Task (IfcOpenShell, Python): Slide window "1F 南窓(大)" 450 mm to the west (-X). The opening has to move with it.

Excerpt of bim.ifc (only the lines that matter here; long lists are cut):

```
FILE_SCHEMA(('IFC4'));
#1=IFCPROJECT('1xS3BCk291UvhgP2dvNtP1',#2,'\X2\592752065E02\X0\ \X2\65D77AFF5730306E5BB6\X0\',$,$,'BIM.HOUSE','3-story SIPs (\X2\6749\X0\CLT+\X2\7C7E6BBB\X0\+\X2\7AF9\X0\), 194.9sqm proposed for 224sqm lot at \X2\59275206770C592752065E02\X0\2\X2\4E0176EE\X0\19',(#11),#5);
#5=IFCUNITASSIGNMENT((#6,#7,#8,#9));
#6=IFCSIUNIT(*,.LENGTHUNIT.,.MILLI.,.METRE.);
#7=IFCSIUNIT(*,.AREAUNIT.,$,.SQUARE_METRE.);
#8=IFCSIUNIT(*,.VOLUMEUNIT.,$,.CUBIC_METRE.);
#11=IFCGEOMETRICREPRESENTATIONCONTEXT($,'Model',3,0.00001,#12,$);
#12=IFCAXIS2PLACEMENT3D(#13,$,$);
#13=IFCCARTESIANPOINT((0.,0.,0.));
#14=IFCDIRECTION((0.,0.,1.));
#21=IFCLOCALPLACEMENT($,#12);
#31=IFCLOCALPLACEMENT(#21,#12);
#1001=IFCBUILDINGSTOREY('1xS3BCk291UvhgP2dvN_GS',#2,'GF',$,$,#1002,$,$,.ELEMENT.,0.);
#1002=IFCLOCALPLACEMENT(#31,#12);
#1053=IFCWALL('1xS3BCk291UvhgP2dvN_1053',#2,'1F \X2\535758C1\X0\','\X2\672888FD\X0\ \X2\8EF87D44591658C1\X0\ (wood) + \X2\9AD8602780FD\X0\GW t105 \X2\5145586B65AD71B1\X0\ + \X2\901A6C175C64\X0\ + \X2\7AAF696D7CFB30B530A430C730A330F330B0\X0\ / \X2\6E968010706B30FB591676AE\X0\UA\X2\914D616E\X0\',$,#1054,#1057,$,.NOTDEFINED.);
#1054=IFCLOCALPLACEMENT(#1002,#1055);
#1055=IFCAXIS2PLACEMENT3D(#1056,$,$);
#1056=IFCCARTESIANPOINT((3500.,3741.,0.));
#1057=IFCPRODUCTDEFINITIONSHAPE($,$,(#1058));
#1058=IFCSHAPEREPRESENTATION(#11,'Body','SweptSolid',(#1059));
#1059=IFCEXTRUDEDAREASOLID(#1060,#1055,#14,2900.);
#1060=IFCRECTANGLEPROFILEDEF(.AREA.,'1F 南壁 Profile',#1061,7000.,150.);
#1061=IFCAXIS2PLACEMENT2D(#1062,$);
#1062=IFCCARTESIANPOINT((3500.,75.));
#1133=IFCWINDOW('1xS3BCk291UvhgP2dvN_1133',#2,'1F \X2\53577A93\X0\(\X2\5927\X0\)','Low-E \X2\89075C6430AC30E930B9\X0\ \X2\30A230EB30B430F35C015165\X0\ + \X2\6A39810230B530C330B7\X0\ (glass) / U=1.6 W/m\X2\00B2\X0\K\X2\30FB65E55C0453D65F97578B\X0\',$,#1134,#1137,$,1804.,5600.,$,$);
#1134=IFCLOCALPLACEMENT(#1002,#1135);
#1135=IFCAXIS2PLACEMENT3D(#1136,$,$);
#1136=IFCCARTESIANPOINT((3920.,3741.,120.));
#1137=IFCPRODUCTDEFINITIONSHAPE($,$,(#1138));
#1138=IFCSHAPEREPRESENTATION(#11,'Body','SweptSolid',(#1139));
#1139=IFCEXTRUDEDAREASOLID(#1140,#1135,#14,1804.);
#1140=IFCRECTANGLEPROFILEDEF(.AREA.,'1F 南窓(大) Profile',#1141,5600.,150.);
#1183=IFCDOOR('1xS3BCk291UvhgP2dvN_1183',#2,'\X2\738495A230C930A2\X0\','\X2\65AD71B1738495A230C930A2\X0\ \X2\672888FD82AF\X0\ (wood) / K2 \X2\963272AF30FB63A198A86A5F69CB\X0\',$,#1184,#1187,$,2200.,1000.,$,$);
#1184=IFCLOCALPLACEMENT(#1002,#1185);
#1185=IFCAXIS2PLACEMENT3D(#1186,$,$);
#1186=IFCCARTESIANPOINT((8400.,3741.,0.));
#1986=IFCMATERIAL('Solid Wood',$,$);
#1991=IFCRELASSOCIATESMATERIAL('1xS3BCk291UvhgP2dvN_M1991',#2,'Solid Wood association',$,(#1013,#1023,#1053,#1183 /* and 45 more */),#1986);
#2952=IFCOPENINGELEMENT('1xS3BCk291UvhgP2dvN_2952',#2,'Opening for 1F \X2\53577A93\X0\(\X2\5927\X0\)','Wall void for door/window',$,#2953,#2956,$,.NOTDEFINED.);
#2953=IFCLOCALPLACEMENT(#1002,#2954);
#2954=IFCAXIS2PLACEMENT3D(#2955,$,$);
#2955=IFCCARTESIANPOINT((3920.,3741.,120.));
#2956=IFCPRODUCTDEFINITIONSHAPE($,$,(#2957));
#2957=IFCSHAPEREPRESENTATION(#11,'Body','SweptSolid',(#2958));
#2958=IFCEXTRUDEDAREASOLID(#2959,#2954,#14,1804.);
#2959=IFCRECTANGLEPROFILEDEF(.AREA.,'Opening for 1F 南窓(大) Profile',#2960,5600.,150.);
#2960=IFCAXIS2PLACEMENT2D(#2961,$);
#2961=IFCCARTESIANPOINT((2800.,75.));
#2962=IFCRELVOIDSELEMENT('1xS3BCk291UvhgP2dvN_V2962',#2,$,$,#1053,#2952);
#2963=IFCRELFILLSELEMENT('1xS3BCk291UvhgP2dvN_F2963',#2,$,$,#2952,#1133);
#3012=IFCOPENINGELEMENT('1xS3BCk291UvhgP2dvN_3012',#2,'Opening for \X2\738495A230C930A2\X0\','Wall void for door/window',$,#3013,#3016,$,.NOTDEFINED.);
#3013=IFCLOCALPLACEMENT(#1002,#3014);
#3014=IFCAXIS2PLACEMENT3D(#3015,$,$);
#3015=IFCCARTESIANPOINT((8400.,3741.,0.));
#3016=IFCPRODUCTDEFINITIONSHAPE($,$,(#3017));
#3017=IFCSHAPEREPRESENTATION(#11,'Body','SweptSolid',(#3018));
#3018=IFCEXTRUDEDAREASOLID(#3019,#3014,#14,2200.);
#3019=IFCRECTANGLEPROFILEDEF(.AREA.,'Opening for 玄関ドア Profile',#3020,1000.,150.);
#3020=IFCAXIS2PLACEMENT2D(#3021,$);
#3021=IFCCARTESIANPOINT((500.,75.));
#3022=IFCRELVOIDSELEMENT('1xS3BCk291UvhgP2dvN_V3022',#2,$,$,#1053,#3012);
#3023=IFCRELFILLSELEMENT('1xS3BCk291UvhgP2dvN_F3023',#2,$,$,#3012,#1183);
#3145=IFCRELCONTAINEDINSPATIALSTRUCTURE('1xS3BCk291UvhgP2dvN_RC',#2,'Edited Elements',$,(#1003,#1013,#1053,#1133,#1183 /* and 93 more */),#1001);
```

```python
import ifcopenshell
import ifcopenshell.api.geometry
import ifcopenshell.util.placement
import ifcopenshell.util.unit

model = ifcopenshell.open("bim.ifc")
unit_scale = ifcopenshell.util.unit.calculate_unit_scale(model)

window = model.by_guid("1xS3BCk291UvhgP2dvN_1133")
opening = window.FillsVoids[0].RelatingOpeningElement
wall = opening.VoidsElements[0].RelatingBuildingElement

wall_matrix = ifcopenshell.util.placement.get_local_placement(wall.ObjectPlacement)
shift = wall_matrix[:3, 0] * -0.45 / unit_scale
before = ifcopenshell.util.placement.get_local_placement(window.ObjectPlacement)[:3, 3].copy()

# The window is not placed relative to its opening, so move both.
for product in (opening, window):
    matrix = ifcopenshell.util.placement.get_local_placement(product.ObjectPlacement)
    matrix[:3, 3] += shift
    ifcopenshell.api.geometry.edit_object_placement(model, product=product, matrix=matrix, is_si=False)

after = ifcopenshell.util.placement.get_local_placement(window.ObjectPlacement)[:3, 3]
print("window moved by", (after - before).round(3) + 0.0)

model.write("bim_v2.ifc")
```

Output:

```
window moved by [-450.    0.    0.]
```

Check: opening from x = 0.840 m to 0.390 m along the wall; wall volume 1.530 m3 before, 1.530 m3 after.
